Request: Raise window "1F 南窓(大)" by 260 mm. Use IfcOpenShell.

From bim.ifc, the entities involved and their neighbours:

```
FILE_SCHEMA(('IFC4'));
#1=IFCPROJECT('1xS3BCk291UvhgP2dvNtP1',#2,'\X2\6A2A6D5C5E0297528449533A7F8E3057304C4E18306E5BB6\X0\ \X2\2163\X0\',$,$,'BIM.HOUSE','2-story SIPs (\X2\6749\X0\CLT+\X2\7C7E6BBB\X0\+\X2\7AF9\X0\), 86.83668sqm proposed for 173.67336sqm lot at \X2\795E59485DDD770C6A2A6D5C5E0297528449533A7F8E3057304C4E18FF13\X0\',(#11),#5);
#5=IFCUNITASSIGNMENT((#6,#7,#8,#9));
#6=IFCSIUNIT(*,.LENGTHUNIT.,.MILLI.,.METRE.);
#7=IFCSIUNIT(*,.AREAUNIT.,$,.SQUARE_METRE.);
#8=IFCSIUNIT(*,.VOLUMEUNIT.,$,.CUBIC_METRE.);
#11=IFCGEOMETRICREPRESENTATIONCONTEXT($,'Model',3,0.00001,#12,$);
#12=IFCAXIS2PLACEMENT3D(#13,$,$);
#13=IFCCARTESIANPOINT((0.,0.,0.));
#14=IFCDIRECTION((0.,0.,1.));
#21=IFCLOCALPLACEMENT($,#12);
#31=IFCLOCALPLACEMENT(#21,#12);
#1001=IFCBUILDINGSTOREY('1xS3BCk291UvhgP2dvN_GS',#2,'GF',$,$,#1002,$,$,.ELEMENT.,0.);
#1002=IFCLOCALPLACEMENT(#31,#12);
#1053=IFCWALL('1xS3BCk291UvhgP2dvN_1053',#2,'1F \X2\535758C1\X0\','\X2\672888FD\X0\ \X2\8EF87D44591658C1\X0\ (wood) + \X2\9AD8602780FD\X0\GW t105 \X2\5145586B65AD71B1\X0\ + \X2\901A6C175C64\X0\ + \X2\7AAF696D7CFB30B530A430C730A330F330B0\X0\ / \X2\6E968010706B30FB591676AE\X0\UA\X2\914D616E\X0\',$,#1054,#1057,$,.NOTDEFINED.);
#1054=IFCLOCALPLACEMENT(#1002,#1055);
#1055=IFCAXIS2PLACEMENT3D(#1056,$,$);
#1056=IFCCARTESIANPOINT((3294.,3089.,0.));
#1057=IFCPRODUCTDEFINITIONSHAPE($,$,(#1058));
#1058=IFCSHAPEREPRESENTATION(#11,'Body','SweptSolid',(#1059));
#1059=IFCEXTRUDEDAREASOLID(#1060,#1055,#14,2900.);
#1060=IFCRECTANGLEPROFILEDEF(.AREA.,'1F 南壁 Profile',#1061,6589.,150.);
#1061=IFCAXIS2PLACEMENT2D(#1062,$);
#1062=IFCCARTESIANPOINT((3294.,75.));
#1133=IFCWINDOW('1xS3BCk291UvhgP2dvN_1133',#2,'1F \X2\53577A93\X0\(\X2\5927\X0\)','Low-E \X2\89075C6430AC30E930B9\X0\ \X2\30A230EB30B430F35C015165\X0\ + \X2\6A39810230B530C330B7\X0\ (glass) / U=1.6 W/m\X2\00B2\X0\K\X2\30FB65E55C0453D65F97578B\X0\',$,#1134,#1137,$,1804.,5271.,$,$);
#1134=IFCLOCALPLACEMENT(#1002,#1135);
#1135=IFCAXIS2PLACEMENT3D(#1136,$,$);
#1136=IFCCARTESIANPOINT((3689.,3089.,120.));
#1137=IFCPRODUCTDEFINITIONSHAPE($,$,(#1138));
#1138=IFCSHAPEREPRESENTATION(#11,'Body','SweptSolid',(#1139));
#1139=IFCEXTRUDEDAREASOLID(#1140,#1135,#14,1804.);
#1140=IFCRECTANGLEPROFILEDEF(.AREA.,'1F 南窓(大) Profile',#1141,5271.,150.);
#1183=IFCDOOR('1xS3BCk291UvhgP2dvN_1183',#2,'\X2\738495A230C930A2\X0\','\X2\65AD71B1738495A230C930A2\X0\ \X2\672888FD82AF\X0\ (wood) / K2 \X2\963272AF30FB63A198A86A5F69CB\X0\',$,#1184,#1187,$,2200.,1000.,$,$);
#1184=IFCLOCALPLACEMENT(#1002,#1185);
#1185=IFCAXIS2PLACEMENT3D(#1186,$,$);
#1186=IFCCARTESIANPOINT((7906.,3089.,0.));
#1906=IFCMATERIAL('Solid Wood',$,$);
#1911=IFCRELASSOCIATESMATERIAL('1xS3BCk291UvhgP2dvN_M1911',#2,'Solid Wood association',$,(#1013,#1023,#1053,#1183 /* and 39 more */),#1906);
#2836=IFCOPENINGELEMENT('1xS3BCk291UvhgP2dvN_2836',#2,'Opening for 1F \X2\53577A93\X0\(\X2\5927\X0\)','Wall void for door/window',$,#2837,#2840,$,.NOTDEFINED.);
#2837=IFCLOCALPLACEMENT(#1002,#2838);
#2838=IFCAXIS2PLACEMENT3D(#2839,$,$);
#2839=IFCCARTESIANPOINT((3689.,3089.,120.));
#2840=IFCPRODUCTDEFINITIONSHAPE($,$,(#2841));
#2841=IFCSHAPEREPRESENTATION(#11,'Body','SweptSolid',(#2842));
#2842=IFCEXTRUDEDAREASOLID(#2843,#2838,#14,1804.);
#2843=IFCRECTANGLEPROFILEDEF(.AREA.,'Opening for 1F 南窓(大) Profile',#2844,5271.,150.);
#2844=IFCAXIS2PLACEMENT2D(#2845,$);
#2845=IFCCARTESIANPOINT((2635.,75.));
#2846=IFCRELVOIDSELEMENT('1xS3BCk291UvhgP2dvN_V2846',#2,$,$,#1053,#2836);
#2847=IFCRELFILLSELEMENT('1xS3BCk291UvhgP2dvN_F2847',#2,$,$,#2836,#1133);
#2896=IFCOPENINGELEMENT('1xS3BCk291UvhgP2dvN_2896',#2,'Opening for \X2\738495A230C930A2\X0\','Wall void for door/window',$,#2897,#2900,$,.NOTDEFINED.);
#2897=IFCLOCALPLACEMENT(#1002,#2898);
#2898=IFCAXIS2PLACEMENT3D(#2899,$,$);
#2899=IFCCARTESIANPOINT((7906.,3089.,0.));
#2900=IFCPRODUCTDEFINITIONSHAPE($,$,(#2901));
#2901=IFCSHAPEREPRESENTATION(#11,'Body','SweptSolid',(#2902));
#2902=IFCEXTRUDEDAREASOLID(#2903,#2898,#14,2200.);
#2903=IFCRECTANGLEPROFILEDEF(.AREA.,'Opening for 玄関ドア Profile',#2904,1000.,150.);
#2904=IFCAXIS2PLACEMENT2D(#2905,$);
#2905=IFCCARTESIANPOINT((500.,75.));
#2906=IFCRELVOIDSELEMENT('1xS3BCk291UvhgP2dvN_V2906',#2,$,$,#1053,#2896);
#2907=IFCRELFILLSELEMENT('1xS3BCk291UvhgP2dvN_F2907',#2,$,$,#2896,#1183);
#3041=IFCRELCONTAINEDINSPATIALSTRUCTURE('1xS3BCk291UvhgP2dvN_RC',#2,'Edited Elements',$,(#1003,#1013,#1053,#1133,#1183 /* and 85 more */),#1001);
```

```python
import numpy as np
import ifcopenshell
import ifcopenshell.api.geometry
import ifcopenshell.util.placement
import ifcopenshell.util.unit

model = ifcopenshell.open("bim.ifc")
unit_scale = ifcopenshell.util.unit.calculate_unit_scale(model)

window = model.by_guid("1xS3BCk291UvhgP2dvN_1133")
opening = window.FillsVoids[0].RelatingOpeningElement
dz = 260.0

shift = np.array([0.0, 0.0, dz])
# The window is not placed relative to its opening, so move both.
for product in (opening, window):
    matrix = ifcopenshell.util.placement.get_local_placement(product.ObjectPlacement)
    matrix[:3, 3] += shift
    ifcopenshell.api.geometry.edit_object_placement(model, product=product, matrix=matrix, is_si=False)

print(f"moved by {dz * unit_scale:+.3f} m")

model.write("bim_v2.ifc")
```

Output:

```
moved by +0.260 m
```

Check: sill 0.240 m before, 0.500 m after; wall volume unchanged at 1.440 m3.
